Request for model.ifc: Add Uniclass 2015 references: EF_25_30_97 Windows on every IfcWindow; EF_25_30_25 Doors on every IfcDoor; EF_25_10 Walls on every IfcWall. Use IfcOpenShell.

First a look at what the model holds.

```python
import ifcopenshell

model = ifcopenshell.open("model.ifc")
print(model.schema)
print("classifications:", [c.Name for c in model.by_type("IfcClassification")])
for ifc_class in ("IfcDoor", "IfcRoof", "IfcStair", "IfcWall", "IfcWindow"):
    print(ifc_class, len(model.by_type(ifc_class)))
```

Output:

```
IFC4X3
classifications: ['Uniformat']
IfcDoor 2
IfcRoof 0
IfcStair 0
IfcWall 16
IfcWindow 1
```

```python
import ifcopenshell
import ifcopenshell.api.classification

model = ifcopenshell.open("model.ifc")

system = ifcopenshell.api.classification.add_classification(model, classification="Uniclass 2015")

codes = {
    "IfcWindow": ("EF_25_30_97", "Windows"),
    "IfcDoor": ("EF_25_30_25", "Doors"),
    "IfcWall": ("EF_25_10", "Walls"),
}
for ifc_class, (code, name) in codes.items():
    products = model.by_type(ifc_class)
    ifcopenshell.api.classification.add_reference(
        model, products=products, classification=system, identification=code, name=name
    )
    print(code, len(products))

model.write("model_edited.ifc")
```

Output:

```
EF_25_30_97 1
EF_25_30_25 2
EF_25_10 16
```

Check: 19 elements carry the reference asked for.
